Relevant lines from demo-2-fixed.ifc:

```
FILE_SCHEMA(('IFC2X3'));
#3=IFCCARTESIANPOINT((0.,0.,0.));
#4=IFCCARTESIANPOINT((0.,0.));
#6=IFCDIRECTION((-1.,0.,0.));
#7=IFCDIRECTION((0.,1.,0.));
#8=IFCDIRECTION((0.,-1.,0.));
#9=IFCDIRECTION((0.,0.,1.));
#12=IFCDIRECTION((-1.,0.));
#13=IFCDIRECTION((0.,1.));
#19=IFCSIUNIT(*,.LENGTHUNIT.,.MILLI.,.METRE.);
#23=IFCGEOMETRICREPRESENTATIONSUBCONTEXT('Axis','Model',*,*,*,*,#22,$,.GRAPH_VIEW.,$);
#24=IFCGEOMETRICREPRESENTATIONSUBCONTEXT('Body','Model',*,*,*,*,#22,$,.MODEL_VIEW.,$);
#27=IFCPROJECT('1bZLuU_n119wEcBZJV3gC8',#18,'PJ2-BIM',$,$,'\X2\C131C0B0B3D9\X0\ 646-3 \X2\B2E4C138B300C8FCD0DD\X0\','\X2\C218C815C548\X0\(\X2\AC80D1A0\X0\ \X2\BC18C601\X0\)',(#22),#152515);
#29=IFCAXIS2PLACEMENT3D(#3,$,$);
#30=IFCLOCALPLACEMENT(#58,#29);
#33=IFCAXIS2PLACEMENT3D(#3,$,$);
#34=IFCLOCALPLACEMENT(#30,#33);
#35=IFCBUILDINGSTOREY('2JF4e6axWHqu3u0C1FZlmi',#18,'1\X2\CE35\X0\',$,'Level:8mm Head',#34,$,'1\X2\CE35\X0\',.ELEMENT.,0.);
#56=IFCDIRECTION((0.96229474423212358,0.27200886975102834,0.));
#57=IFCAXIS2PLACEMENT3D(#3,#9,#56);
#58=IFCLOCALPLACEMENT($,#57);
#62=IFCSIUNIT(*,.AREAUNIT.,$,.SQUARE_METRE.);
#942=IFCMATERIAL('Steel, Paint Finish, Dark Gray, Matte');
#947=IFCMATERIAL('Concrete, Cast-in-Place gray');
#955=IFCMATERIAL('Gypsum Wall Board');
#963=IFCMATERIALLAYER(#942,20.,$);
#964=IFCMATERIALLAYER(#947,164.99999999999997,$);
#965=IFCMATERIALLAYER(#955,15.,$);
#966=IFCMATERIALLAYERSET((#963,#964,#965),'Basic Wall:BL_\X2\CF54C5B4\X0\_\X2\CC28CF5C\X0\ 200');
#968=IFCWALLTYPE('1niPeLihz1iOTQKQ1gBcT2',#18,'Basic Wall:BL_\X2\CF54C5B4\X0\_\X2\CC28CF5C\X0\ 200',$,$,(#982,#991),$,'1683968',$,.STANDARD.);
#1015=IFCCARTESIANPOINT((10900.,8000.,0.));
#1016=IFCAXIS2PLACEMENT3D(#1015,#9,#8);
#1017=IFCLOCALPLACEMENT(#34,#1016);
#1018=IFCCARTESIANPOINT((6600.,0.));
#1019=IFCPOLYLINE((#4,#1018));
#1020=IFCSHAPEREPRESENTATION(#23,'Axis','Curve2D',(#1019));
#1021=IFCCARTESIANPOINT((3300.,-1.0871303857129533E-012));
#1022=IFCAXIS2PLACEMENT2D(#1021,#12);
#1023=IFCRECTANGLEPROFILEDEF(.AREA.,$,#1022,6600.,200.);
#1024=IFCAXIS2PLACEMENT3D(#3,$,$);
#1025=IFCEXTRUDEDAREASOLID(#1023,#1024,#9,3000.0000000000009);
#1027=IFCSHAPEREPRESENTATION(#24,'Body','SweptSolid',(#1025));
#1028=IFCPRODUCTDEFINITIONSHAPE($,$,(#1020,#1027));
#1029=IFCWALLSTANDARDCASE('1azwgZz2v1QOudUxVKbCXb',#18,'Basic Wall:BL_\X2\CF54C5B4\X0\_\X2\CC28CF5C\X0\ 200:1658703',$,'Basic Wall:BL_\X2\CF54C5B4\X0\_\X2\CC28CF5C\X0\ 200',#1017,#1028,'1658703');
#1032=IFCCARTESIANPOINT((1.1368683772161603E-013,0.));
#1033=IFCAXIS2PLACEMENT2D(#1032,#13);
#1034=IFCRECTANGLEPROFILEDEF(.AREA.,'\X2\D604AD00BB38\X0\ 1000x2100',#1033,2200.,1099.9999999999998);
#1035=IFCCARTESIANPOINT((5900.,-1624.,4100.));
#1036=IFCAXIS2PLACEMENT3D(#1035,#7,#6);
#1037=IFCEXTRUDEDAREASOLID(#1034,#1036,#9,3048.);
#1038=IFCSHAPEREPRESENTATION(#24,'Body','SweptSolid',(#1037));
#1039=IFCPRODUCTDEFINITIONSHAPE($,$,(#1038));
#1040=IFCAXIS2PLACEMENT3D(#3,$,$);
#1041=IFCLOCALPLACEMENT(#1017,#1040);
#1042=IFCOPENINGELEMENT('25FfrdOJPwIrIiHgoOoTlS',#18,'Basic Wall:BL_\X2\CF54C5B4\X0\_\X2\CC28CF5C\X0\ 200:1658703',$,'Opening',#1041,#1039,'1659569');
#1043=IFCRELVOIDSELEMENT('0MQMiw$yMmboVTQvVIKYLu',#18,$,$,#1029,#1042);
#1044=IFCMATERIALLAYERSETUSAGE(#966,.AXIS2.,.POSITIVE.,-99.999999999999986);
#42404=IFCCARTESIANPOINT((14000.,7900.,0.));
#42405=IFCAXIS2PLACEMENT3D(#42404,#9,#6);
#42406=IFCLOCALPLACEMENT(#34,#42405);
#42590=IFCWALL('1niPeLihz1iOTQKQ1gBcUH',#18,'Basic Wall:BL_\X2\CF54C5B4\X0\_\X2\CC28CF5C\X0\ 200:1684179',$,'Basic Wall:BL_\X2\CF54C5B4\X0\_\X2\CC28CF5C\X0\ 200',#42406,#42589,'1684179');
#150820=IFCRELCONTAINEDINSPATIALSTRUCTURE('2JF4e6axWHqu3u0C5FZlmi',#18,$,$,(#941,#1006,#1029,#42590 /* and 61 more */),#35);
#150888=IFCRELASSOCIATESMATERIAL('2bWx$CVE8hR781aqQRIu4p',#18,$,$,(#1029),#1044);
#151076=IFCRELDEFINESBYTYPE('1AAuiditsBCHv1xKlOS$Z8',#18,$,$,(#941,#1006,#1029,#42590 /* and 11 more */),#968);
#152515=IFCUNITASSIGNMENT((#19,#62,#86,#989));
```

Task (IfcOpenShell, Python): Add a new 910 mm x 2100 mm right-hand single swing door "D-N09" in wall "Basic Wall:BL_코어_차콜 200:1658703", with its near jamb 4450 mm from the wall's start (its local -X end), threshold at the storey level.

```python
import numpy as np
import ifcopenshell
import ifcopenshell.api.feature
import ifcopenshell.api.geometry
import ifcopenshell.api.root
import ifcopenshell.api.spatial
import ifcopenshell.api.type
import ifcopenshell.geom
import ifcopenshell.util.element
import ifcopenshell.util.placement
import ifcopenshell.util.representation
import ifcopenshell.util.shape
import ifcopenshell.util.unit

model = ifcopenshell.open("demo-2-fixed.ifc")
unit_scale = ifcopenshell.util.unit.calculate_unit_scale(model)
settings = ifcopenshell.geom.settings()


def volume(element):
    """Net volume in cubic metres, openings subtracted."""
    shape = ifcopenshell.geom.create_shape(settings, element)
    return ifcopenshell.util.shape.get_volume(shape.geometry)


wall = model.by_guid("1azwgZz2v1QOudUxVKbCXb")
storey = ifcopenshell.util.element.get_container(wall, ifc_class="IfcBuildingStorey")
context = ifcopenshell.util.representation.get_context(model, "Model", "Body", "MODEL_VIEW")
before = volume(wall)

width, height, from_end, sill = 0.91, 2.1, 4.45, 0.0  # metres

# The wall runs along its own X axis, and the end named is its -X end.
wall_shape = ifcopenshell.geom.create_shape(settings, wall)
x, y, z = ifcopenshell.util.shape.get_vertices(wall_shape.geometry).T
start = x.min() + from_end
face, thickness = float(y.min()), float(y.max() - y.min())
wall_matrix = ifcopenshell.util.placement.get_local_placement(wall.ObjectPlacement)
level = ifcopenshell.util.placement.get_local_placement(storey.ObjectPlacement)[2, 3]


def in_wall(x, y):
    """Placement at x, y metres in the wall's axes, at sill height."""
    matrix = wall_matrix.copy()
    matrix[:, 3] = wall_matrix @ np.array([x / unit_scale, y / unit_scale, 0.0, 1.0])
    matrix[2, 3] = level + sill / unit_scale
    return matrix


# Opening: a box that overshoots both wall faces by 50 mm.
opening = ifcopenshell.api.root.create_entity(model, ifc_class="IfcOpeningElement")
box = ifcopenshell.api.geometry.add_wall_representation(
    model, context=context, length=width, height=height, thickness=thickness + 0.1
)
ifcopenshell.api.geometry.assign_representation(model, product=opening, representation=box)
ifcopenshell.api.geometry.edit_object_placement(model, product=opening, matrix=in_wall(start, face - 0.05), is_si=False)
ifcopenshell.api.feature.add_feature(model, feature=opening, element=wall)

door = ifcopenshell.api.root.create_entity(model, ifc_class="IfcDoor", name="D-N09")
door.OverallWidth, door.OverallHeight = width / unit_scale, height / unit_scale
body = ifcopenshell.api.geometry.add_door_representation(
    model,
    context=context,
    overall_width=door.OverallWidth,
    overall_height=door.OverallHeight,
    operation_type="SINGLE_SWING_RIGHT",
    lining_properties={"LiningDepth": thickness / unit_scale, "ThresholdDepth": thickness / unit_scale},
)
ifcopenshell.api.geometry.assign_representation(model, product=door, representation=body)
ifcopenshell.api.spatial.assign_container(model, products=[door], relating_structure=storey)
fills = ifcopenshell.api.feature.add_filling(model, opening=opening, element=door)
fills.OwnerHistory = door.OwnerHistory  # required in IFC2X3

# IFC2X3 keeps the operation on the door style.
style = ifcopenshell.api.root.create_entity(model, ifc_class="IfcDoorStyle", name="D-N09")
style.OperationType, style.ConstructionType = "SINGLE_SWING_RIGHT", "NOTDEFINED"
style.ParameterTakesPrecedence = style.Sizeable = False
ifcopenshell.api.type.assign_type(model, related_objects=[door], relating_type=style)

# The lining spans the wall, so the door starts at the wall face.
ifcopenshell.api.geometry.edit_object_placement(model, product=door, matrix=in_wall(start, face), is_si=False)

after = volume(wall)

print(f"wall volume {before:.3f} -> {after:.3f} m3")

model.write("demo-2-fixed_v2.ifc")
```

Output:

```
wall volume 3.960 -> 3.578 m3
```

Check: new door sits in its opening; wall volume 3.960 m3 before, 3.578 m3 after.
